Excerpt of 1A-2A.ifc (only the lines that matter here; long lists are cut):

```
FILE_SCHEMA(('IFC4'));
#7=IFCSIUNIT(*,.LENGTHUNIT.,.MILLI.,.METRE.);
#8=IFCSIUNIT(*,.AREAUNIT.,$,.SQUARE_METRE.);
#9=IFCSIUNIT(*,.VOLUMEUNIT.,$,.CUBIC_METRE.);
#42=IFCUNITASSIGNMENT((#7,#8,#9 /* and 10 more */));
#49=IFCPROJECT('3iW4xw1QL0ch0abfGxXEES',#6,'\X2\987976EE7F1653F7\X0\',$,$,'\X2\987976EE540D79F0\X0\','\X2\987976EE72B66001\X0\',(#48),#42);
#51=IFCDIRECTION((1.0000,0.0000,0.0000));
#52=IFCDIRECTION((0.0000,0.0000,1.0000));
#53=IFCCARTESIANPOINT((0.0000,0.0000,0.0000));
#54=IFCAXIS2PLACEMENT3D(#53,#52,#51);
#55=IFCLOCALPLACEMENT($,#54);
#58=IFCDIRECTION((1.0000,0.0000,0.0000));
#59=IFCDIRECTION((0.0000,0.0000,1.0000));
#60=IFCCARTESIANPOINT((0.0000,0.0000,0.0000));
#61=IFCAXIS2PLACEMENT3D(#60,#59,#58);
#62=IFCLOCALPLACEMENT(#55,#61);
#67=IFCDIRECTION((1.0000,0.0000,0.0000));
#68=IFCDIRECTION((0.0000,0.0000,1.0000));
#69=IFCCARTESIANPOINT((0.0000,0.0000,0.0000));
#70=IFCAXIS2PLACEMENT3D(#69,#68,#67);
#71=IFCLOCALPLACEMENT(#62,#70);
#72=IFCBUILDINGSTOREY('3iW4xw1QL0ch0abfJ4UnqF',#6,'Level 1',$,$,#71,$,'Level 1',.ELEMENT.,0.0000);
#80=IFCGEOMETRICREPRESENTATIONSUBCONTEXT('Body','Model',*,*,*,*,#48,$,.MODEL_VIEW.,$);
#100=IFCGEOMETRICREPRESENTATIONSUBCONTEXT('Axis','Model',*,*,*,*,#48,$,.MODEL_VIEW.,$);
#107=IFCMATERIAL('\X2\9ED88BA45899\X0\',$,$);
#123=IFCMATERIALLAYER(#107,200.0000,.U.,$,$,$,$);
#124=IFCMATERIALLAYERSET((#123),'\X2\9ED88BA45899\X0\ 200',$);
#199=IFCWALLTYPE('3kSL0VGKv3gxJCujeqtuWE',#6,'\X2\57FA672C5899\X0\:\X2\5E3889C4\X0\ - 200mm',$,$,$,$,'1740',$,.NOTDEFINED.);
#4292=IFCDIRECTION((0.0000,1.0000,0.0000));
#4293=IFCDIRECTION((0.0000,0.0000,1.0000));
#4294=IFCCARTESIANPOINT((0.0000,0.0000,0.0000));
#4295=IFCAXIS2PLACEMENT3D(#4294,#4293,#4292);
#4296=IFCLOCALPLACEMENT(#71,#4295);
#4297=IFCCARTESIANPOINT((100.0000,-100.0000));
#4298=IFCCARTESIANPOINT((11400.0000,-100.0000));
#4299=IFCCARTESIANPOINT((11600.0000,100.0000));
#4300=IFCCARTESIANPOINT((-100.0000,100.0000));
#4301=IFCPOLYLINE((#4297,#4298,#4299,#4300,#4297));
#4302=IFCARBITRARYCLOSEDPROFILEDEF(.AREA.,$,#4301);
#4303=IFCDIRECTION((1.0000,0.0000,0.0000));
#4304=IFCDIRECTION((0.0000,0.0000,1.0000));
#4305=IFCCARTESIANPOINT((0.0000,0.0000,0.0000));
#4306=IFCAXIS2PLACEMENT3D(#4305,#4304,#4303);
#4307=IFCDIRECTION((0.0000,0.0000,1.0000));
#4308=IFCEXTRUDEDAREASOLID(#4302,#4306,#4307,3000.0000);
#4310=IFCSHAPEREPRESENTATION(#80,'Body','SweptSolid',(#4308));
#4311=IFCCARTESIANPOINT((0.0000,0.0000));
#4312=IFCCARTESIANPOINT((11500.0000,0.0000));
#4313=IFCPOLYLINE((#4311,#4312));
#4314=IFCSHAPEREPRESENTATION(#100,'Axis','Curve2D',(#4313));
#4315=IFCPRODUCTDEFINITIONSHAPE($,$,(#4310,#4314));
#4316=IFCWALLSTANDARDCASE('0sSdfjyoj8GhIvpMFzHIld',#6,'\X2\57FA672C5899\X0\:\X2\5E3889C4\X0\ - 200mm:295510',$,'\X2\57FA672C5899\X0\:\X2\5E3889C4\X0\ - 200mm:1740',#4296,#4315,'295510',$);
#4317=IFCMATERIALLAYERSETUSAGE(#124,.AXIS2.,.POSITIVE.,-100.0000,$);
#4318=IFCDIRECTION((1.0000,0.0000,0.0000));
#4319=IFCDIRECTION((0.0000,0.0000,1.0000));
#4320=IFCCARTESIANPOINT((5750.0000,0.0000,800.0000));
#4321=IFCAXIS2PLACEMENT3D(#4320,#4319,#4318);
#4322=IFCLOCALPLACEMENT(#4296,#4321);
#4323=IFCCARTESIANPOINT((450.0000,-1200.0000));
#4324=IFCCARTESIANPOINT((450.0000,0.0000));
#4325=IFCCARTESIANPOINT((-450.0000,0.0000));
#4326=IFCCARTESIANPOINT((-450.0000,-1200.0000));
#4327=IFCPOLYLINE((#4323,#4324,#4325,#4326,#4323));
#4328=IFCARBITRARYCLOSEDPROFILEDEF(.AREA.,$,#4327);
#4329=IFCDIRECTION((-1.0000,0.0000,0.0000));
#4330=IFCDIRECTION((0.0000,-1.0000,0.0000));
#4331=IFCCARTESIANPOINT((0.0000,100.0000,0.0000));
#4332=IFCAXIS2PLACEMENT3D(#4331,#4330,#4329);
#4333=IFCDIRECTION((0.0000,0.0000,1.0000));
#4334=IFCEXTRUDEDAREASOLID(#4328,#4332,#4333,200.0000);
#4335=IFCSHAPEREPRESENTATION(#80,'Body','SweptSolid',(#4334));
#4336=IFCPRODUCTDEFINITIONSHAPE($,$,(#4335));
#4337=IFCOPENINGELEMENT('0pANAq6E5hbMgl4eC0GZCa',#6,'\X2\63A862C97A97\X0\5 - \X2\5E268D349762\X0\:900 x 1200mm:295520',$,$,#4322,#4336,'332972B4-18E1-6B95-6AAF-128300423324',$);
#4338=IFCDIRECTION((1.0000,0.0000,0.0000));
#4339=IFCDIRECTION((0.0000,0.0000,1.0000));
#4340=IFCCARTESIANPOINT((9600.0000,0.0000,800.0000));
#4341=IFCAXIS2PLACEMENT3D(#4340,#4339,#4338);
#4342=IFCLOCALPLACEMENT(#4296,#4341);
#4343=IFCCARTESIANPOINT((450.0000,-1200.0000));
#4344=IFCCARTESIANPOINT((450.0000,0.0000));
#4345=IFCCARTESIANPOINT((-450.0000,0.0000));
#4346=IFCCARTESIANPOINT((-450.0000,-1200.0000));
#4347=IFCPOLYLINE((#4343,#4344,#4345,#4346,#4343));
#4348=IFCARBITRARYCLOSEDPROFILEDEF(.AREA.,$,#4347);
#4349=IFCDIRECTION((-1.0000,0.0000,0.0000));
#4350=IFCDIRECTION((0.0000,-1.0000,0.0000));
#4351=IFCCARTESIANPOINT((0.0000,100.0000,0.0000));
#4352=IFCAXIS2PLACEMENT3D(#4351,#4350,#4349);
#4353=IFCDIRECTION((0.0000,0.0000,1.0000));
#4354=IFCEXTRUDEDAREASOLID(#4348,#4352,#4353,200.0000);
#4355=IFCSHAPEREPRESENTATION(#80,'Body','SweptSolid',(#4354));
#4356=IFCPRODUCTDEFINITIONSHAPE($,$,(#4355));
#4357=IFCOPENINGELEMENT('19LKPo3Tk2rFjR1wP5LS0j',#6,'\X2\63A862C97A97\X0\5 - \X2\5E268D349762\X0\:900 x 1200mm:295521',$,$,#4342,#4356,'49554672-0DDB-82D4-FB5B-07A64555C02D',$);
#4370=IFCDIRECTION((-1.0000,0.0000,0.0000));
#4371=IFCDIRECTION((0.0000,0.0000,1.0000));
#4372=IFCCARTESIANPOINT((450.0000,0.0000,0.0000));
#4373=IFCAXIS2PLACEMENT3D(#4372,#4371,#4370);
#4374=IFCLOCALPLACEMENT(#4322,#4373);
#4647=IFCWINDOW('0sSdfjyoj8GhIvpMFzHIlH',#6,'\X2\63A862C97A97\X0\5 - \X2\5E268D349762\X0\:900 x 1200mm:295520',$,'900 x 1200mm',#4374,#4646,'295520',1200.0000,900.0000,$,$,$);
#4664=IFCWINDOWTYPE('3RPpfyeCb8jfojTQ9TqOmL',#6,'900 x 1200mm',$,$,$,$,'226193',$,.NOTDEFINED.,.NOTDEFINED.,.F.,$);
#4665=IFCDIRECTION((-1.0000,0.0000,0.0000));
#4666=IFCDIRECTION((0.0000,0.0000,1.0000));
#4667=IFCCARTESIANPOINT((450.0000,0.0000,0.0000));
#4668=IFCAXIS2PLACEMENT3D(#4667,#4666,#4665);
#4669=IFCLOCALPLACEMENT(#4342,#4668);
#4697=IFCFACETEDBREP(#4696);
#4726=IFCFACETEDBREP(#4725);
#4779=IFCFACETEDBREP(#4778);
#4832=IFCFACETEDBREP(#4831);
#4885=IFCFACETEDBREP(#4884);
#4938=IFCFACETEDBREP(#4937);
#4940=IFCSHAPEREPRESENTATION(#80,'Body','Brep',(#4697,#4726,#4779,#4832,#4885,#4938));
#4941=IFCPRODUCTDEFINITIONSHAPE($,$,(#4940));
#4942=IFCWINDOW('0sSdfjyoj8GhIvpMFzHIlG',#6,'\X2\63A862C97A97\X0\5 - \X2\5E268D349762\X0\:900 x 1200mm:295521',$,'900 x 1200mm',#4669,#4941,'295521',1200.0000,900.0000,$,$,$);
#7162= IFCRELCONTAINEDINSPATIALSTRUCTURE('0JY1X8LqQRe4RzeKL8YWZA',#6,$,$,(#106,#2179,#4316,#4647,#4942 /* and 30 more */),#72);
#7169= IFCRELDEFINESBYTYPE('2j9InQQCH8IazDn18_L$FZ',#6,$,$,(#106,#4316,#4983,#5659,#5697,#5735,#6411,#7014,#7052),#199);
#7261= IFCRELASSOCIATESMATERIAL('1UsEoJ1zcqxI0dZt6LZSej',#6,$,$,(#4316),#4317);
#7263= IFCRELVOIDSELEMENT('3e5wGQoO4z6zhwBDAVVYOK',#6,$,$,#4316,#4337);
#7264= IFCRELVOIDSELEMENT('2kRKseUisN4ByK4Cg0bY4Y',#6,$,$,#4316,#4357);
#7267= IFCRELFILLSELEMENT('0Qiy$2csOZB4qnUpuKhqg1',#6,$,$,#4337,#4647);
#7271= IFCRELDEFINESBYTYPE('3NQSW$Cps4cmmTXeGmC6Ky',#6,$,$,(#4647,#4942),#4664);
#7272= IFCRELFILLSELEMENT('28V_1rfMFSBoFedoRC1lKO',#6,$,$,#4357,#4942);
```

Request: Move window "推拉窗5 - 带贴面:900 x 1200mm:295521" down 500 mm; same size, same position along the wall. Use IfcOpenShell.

```python
import numpy as np
import ifcopenshell
import ifcopenshell.api.geometry
import ifcopenshell.util.placement
import ifcopenshell.util.unit

model = ifcopenshell.open("1A-2A.ifc")
unit_scale = ifcopenshell.util.unit.calculate_unit_scale(model)

window = model.by_guid("0sSdfjyoj8GhIvpMFzHIlG")
opening = window.FillsVoids[0].RelatingOpeningElement
dz = -0.5 / unit_scale

shift = np.array([0.0, 0.0, dz])
# The window is placed relative to its opening, so it follows when the opening moves.
matrix = ifcopenshell.util.placement.get_local_placement(opening.ObjectPlacement)
matrix[:3, 3] += shift
ifcopenshell.api.geometry.edit_object_placement(
    model, product=opening, matrix=matrix, is_si=False, should_transform_children=True
)

print(f"moved by {dz * unit_scale:+.3f} m")

model.write("1A-2A-out.ifc")
```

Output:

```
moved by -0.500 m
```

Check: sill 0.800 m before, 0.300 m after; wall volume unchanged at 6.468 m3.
